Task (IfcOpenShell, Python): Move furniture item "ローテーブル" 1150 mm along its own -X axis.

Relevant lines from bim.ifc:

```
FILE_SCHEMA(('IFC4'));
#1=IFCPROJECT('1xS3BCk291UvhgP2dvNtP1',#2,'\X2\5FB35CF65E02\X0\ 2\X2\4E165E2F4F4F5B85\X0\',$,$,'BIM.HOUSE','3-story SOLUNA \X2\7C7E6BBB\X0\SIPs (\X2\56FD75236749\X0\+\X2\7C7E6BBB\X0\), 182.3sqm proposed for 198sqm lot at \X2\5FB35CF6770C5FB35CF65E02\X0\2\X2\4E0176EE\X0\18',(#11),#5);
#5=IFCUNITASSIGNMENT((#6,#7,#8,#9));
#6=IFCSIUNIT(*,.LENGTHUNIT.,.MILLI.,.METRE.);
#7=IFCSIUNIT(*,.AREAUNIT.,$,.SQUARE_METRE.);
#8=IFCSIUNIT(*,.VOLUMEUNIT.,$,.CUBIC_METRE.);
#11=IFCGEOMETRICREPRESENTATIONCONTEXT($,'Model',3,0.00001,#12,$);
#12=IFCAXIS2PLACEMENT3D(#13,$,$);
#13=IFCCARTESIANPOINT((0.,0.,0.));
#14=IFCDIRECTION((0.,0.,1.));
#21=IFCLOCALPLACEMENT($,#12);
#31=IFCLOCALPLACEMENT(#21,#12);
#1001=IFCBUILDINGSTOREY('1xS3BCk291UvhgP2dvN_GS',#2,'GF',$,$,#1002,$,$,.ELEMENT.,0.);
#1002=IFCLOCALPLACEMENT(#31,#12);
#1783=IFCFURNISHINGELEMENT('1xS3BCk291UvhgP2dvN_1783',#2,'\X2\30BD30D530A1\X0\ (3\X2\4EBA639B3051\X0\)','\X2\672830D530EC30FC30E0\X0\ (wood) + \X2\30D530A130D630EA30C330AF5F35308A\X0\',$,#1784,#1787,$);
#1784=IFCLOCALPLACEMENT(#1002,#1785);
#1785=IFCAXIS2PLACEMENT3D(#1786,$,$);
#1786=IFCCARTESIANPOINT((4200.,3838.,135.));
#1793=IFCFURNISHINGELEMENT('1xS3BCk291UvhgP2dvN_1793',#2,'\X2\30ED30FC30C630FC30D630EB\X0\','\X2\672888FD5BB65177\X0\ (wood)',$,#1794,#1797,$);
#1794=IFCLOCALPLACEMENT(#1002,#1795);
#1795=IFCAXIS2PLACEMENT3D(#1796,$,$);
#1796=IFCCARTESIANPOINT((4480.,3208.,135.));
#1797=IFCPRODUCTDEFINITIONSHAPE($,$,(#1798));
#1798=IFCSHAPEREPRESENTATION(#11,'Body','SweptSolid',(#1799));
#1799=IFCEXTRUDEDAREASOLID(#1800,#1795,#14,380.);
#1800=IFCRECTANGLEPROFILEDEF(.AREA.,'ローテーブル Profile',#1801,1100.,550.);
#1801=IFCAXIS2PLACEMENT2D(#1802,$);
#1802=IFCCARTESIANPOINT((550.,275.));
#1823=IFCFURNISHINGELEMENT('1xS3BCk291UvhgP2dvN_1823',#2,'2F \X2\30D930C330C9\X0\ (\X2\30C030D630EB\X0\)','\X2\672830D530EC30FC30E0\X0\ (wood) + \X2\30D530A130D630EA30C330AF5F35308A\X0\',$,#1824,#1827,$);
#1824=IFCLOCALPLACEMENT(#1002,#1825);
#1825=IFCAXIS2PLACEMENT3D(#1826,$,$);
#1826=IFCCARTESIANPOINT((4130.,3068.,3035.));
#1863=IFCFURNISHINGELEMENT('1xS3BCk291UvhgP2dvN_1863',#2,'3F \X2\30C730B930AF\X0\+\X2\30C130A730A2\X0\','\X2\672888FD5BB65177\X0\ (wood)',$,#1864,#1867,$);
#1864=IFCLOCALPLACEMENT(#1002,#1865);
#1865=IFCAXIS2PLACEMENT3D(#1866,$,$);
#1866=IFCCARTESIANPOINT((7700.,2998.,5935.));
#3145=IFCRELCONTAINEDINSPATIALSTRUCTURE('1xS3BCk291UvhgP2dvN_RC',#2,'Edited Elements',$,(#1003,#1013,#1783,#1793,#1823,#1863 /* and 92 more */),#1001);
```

```python
import ifcopenshell
import ifcopenshell.api.geometry
import ifcopenshell.util.placement

model = ifcopenshell.open("bim.ifc")

item = model.by_guid("1xS3BCk291UvhgP2dvN_1793")
matrix = ifcopenshell.util.placement.get_local_placement(item.ObjectPlacement)
matrix[:3, 3] -= matrix[:3, 0] * 1150.0
ifcopenshell.api.geometry.edit_object_placement(model, product=item, matrix=matrix, is_si=False)

print(ifcopenshell.util.placement.get_local_placement(item.ObjectPlacement).round(3) + 0.0)

model.write("bim_updated.ifc")
```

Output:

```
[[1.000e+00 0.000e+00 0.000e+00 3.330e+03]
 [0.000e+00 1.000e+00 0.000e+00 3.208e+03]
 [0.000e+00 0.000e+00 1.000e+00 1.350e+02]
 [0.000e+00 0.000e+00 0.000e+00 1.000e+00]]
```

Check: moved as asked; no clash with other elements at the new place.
